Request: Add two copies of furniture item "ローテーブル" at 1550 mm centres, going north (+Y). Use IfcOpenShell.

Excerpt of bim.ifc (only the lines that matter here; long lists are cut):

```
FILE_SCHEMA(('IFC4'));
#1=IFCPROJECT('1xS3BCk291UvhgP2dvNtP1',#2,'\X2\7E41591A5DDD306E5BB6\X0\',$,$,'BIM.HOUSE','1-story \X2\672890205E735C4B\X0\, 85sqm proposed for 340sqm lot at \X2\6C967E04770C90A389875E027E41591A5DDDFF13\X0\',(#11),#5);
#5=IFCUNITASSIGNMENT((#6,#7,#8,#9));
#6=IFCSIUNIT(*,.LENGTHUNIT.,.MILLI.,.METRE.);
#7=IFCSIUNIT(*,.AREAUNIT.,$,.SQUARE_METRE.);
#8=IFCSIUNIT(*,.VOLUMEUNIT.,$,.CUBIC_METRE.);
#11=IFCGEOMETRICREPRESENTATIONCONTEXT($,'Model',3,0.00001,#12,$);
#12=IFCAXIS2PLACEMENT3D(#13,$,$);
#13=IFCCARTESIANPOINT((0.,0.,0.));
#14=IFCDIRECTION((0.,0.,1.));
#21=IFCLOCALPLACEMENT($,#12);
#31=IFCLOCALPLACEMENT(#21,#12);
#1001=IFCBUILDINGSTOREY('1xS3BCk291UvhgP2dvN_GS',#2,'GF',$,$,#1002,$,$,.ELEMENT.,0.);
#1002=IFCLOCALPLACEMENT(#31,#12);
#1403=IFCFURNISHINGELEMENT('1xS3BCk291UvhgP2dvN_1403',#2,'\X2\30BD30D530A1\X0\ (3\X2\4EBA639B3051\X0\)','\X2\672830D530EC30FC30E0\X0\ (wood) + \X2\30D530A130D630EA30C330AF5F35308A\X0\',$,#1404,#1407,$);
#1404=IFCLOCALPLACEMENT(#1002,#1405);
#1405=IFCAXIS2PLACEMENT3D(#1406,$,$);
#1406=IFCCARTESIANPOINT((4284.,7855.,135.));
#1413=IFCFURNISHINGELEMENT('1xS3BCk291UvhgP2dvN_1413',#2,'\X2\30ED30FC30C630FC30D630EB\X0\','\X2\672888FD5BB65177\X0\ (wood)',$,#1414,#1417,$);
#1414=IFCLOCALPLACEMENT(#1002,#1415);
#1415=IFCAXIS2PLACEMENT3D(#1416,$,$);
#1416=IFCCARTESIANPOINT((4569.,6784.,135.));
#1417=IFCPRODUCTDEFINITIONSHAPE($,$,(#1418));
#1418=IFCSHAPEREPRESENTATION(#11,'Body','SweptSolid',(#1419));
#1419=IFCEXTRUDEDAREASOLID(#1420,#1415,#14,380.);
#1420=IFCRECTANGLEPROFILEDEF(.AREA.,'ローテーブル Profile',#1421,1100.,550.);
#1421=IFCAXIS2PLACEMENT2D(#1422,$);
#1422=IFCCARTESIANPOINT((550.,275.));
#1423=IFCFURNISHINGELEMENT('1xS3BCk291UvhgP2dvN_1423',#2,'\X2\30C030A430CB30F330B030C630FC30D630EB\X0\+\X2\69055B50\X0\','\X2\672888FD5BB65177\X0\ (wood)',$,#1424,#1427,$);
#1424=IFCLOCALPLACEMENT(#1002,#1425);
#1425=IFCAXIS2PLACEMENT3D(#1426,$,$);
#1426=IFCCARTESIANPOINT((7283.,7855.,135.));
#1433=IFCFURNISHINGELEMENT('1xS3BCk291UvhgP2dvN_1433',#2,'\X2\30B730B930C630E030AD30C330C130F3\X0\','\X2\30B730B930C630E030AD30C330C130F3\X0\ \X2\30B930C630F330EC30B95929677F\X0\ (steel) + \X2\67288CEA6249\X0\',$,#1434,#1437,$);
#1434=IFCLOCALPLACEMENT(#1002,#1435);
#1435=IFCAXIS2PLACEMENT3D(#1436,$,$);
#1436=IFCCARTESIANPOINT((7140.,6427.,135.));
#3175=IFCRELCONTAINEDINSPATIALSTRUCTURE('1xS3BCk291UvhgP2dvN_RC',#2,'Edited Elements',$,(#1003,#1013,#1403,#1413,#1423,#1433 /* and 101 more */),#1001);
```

```python
import numpy as np
import ifcopenshell
import ifcopenshell.api.geometry
import ifcopenshell.api.root
import ifcopenshell.util.element
import ifcopenshell.util.placement
import ifcopenshell.util.unit

model = ifcopenshell.open("bim.ifc")
unit_scale = ifcopenshell.util.unit.calculate_unit_scale(model)


def reuse_history(source, copy):
    """copy_class also copies each property set's owner history, people and application; keep the originals."""
    for rel in copy.IsDefinedBy:
        if rel.is_a("IfcRelDefinesByProperties") and (history := rel.RelatingPropertyDefinition.OwnerHistory):
            rel.RelatingPropertyDefinition.OwnerHistory = source.OwnerHistory
            ifcopenshell.util.element.remove_deep2(model, history)


source = model.by_guid("1xS3BCk291UvhgP2dvN_1413")
base = ifcopenshell.util.placement.get_local_placement(source.ObjectPlacement)
step = np.array([0.0, 1.0, 0.0]) * 1.55 / unit_scale

for i in range(1, 3):
    copy = ifcopenshell.api.root.copy_class(model, product=source)
    copy.Representation = ifcopenshell.util.element.copy_deep(
        model, source.Representation, exclude=["IfcGeometricRepresentationContext", "IfcRepresentationMap"]
    )
    reuse_history(source, copy)
    matrix = base.copy()
    matrix[:3, 3] += i * step
    print("added at", matrix[:3, 3].round(3) + 0.0)
    ifcopenshell.api.geometry.edit_object_placement(model, product=copy, matrix=matrix, is_si=False)

model.write("bim_edited.ifc")
```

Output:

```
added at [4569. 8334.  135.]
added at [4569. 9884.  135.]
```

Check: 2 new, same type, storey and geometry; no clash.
